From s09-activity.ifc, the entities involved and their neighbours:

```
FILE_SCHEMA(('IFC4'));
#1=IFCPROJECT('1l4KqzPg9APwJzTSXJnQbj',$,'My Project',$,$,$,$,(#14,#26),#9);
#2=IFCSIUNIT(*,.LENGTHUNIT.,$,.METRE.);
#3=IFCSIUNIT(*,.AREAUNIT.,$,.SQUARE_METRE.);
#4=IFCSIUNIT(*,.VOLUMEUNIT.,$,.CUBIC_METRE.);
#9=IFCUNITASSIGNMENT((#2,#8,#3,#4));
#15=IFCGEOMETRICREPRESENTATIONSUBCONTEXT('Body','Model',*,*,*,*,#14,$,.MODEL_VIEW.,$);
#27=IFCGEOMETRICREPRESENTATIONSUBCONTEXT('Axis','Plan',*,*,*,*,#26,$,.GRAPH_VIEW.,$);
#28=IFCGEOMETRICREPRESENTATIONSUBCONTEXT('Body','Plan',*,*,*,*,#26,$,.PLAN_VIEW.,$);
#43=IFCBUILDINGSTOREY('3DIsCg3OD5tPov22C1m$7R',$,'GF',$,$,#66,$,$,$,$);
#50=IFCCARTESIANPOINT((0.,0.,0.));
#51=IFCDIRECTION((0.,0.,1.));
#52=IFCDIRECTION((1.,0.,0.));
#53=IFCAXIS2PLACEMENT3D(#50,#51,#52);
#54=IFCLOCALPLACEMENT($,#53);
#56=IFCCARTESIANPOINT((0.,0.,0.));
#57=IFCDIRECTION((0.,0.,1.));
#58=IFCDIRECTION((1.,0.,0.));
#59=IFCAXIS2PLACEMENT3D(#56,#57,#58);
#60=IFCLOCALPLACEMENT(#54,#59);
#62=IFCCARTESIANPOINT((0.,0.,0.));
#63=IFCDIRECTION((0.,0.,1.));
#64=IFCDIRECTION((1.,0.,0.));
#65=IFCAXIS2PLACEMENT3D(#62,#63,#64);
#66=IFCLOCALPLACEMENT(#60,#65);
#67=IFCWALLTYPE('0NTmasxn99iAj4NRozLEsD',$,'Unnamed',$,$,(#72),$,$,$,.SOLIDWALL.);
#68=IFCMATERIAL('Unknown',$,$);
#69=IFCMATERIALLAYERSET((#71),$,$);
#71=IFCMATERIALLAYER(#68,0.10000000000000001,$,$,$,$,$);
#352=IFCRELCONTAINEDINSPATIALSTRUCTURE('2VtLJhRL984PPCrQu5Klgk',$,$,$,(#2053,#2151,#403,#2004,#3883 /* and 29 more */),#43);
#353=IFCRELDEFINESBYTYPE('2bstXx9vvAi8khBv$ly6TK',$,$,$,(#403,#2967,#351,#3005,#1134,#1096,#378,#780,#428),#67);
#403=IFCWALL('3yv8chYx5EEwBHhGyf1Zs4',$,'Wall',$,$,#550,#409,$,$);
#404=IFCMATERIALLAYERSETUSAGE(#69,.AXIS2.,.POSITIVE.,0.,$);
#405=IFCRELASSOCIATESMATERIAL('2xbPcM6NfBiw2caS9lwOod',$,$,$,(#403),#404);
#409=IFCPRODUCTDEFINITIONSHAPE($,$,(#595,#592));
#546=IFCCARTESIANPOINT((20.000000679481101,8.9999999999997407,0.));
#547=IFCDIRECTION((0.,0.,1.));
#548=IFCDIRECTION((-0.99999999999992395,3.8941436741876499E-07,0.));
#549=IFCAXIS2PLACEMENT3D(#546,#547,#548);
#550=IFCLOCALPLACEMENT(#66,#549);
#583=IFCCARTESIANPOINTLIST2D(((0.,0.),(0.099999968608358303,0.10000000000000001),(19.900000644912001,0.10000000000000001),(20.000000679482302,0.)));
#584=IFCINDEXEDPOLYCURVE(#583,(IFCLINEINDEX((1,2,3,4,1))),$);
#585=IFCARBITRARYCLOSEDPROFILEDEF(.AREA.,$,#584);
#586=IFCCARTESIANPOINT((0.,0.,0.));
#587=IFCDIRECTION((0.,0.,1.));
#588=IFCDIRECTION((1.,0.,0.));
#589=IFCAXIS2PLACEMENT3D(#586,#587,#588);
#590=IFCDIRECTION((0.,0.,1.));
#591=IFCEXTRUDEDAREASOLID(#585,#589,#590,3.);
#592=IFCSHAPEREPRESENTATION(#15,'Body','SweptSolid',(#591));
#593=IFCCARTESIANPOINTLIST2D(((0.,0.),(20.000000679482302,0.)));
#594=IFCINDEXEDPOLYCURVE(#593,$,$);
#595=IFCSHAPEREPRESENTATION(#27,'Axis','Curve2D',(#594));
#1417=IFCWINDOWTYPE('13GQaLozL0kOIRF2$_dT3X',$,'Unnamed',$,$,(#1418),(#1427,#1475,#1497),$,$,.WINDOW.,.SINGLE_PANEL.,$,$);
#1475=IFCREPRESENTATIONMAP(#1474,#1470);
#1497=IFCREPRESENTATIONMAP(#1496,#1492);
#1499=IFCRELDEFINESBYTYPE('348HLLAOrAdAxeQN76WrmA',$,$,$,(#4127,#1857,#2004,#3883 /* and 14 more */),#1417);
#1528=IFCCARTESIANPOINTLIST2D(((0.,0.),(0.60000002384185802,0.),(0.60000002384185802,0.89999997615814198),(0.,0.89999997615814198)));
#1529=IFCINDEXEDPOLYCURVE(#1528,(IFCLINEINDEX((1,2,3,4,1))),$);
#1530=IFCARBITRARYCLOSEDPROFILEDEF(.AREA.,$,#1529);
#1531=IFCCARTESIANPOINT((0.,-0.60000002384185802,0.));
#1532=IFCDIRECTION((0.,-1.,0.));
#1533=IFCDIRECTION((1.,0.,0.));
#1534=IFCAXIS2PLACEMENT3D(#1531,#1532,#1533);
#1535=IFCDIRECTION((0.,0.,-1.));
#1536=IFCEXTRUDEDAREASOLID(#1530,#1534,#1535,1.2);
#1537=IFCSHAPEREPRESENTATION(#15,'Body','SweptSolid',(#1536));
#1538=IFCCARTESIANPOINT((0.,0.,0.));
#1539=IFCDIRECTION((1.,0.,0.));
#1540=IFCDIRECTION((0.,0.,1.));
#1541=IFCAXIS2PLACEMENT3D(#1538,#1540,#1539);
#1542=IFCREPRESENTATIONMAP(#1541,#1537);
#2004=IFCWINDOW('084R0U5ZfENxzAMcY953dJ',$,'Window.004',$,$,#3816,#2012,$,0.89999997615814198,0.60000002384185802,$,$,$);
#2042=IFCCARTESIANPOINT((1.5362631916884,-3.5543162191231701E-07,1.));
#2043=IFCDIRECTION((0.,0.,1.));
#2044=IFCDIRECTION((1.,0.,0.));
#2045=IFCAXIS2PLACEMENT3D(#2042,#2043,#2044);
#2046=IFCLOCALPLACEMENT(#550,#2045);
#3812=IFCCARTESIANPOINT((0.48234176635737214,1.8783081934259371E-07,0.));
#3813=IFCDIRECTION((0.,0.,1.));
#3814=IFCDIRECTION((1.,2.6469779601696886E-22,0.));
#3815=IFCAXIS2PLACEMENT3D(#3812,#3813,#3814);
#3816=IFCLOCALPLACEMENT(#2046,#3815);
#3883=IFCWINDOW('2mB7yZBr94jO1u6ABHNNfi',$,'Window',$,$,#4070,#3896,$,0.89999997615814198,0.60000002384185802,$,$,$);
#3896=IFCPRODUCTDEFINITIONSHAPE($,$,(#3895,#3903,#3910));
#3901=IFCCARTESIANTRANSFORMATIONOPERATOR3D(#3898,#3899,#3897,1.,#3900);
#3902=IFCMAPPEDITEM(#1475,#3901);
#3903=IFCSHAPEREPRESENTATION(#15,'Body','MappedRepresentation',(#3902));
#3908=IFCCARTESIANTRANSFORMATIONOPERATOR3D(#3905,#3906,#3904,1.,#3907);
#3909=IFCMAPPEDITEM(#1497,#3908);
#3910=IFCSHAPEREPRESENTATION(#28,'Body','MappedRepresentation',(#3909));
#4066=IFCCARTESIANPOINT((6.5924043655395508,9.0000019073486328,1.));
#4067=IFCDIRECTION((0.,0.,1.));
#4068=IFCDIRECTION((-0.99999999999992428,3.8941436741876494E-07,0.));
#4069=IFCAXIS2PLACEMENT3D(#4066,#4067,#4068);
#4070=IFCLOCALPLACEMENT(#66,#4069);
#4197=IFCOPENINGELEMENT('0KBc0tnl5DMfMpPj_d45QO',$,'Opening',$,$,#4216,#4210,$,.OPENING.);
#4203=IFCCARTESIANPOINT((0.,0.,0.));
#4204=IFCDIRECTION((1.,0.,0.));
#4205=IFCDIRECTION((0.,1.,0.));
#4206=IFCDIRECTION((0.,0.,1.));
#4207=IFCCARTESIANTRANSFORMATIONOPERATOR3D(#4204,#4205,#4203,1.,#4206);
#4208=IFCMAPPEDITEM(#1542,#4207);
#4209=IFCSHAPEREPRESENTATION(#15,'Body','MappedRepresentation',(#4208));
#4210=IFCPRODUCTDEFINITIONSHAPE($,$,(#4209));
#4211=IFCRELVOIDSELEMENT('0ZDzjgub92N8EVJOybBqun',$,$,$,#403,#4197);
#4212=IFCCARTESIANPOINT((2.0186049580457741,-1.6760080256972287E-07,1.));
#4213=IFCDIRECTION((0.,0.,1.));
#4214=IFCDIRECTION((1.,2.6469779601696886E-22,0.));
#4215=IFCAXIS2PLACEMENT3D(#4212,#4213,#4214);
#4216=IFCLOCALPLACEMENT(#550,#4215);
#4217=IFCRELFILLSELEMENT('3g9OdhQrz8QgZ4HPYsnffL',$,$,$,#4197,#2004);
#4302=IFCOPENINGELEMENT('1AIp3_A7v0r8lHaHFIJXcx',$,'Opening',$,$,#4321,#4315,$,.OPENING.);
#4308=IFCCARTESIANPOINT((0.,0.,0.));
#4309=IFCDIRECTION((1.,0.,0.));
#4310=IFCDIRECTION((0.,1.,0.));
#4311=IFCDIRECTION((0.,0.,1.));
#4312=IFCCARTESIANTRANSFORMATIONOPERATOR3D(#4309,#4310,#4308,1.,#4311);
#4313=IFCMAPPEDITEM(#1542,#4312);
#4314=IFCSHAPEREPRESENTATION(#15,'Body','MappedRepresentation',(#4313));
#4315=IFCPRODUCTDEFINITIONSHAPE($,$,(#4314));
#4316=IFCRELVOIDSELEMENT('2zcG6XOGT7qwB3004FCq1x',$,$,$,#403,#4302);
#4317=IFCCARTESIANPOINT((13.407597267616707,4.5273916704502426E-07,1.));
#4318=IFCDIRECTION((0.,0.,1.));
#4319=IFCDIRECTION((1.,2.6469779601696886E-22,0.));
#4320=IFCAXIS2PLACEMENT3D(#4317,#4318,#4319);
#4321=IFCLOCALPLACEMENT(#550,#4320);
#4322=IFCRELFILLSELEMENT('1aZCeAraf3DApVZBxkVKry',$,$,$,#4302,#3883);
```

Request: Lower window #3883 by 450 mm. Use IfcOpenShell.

```python
import numpy as np
import ifcopenshell
import ifcopenshell.api.geometry
import ifcopenshell.util.placement
import ifcopenshell.util.unit

model = ifcopenshell.open("s09-activity.ifc")
unit_scale = ifcopenshell.util.unit.calculate_unit_scale(model)

window = model.by_id(3883)
opening = window.FillsVoids[0].RelatingOpeningElement
dz = -0.45 / unit_scale

shift = np.array([0.0, 0.0, dz])
# The window is not placed relative to its opening, so move both.
for product in (opening, window):
    matrix = ifcopenshell.util.placement.get_local_placement(product.ObjectPlacement)
    matrix[:3, 3] += shift
    ifcopenshell.api.geometry.edit_object_placement(model, product=product, matrix=matrix, is_si=False)

print(f"moved by {dz * unit_scale:+.3f} m")

model.write("s09-activity_updated.ifc")
```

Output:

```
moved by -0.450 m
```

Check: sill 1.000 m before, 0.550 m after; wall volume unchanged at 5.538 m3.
